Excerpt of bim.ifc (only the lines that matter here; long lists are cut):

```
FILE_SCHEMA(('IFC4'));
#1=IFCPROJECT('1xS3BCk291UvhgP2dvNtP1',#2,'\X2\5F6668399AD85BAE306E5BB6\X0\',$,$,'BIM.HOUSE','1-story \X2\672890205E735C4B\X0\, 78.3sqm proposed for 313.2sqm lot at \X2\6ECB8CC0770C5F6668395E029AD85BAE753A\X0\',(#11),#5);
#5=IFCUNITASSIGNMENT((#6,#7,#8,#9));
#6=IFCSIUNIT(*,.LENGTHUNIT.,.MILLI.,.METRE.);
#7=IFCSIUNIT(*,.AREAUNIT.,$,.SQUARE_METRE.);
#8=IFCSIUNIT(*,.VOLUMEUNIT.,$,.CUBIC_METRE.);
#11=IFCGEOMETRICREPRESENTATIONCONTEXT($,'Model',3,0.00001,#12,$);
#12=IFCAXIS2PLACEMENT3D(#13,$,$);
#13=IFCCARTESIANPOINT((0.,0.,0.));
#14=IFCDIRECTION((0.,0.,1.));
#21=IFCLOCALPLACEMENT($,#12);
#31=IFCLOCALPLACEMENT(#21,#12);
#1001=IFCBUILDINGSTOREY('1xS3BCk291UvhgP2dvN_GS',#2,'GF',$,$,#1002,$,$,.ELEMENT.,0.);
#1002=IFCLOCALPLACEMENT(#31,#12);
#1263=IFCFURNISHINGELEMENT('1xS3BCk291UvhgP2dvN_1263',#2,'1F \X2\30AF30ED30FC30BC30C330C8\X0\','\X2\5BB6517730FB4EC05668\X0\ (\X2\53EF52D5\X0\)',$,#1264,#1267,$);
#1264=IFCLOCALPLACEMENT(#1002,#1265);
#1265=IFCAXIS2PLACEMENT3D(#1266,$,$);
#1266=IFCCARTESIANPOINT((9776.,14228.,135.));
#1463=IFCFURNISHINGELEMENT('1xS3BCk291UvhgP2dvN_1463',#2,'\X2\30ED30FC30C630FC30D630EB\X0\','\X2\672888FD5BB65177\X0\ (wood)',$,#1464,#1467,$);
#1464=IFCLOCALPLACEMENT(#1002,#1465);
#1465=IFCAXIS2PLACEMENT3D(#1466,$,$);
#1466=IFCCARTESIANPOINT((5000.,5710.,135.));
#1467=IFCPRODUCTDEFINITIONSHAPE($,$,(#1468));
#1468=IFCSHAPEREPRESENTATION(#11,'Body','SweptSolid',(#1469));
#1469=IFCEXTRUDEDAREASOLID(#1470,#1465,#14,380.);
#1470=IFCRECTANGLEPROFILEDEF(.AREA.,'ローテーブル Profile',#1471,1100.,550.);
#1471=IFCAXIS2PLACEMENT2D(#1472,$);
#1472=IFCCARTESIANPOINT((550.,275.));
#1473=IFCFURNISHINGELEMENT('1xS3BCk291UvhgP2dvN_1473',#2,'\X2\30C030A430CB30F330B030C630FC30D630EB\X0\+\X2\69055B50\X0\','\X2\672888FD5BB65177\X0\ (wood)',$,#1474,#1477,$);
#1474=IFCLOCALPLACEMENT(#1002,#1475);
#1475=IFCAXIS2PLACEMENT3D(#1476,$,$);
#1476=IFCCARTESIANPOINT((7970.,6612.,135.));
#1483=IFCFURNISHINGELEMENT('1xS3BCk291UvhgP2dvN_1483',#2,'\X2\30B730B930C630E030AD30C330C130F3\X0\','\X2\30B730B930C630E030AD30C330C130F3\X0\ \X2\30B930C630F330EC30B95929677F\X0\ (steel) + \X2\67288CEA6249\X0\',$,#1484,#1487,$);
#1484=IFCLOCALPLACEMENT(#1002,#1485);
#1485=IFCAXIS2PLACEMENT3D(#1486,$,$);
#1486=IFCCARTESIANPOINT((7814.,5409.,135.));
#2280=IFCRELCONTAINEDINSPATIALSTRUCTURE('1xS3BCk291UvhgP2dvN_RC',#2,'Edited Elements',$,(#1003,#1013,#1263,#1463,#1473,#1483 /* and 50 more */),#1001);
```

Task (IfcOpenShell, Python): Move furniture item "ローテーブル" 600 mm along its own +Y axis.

```python
import ifcopenshell
import ifcopenshell.api.geometry
import ifcopenshell.util.placement
import ifcopenshell.util.unit

model = ifcopenshell.open("bim.ifc")
unit_scale = ifcopenshell.util.unit.calculate_unit_scale(model)

item = model.by_guid("1xS3BCk291UvhgP2dvN_1463")
matrix = ifcopenshell.util.placement.get_local_placement(item.ObjectPlacement)
matrix[:3, 3] += matrix[:3, 1] * 0.6 / unit_scale
ifcopenshell.api.geometry.edit_object_placement(model, product=item, matrix=matrix, is_si=False)

print(ifcopenshell.util.placement.get_local_placement(item.ObjectPlacement).round(3) + 0.0)

model.write("bim_v2.ifc")
```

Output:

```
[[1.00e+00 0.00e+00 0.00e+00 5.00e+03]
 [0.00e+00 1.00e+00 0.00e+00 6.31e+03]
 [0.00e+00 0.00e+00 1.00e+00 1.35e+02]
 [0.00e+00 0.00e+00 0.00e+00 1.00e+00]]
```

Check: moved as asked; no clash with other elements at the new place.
